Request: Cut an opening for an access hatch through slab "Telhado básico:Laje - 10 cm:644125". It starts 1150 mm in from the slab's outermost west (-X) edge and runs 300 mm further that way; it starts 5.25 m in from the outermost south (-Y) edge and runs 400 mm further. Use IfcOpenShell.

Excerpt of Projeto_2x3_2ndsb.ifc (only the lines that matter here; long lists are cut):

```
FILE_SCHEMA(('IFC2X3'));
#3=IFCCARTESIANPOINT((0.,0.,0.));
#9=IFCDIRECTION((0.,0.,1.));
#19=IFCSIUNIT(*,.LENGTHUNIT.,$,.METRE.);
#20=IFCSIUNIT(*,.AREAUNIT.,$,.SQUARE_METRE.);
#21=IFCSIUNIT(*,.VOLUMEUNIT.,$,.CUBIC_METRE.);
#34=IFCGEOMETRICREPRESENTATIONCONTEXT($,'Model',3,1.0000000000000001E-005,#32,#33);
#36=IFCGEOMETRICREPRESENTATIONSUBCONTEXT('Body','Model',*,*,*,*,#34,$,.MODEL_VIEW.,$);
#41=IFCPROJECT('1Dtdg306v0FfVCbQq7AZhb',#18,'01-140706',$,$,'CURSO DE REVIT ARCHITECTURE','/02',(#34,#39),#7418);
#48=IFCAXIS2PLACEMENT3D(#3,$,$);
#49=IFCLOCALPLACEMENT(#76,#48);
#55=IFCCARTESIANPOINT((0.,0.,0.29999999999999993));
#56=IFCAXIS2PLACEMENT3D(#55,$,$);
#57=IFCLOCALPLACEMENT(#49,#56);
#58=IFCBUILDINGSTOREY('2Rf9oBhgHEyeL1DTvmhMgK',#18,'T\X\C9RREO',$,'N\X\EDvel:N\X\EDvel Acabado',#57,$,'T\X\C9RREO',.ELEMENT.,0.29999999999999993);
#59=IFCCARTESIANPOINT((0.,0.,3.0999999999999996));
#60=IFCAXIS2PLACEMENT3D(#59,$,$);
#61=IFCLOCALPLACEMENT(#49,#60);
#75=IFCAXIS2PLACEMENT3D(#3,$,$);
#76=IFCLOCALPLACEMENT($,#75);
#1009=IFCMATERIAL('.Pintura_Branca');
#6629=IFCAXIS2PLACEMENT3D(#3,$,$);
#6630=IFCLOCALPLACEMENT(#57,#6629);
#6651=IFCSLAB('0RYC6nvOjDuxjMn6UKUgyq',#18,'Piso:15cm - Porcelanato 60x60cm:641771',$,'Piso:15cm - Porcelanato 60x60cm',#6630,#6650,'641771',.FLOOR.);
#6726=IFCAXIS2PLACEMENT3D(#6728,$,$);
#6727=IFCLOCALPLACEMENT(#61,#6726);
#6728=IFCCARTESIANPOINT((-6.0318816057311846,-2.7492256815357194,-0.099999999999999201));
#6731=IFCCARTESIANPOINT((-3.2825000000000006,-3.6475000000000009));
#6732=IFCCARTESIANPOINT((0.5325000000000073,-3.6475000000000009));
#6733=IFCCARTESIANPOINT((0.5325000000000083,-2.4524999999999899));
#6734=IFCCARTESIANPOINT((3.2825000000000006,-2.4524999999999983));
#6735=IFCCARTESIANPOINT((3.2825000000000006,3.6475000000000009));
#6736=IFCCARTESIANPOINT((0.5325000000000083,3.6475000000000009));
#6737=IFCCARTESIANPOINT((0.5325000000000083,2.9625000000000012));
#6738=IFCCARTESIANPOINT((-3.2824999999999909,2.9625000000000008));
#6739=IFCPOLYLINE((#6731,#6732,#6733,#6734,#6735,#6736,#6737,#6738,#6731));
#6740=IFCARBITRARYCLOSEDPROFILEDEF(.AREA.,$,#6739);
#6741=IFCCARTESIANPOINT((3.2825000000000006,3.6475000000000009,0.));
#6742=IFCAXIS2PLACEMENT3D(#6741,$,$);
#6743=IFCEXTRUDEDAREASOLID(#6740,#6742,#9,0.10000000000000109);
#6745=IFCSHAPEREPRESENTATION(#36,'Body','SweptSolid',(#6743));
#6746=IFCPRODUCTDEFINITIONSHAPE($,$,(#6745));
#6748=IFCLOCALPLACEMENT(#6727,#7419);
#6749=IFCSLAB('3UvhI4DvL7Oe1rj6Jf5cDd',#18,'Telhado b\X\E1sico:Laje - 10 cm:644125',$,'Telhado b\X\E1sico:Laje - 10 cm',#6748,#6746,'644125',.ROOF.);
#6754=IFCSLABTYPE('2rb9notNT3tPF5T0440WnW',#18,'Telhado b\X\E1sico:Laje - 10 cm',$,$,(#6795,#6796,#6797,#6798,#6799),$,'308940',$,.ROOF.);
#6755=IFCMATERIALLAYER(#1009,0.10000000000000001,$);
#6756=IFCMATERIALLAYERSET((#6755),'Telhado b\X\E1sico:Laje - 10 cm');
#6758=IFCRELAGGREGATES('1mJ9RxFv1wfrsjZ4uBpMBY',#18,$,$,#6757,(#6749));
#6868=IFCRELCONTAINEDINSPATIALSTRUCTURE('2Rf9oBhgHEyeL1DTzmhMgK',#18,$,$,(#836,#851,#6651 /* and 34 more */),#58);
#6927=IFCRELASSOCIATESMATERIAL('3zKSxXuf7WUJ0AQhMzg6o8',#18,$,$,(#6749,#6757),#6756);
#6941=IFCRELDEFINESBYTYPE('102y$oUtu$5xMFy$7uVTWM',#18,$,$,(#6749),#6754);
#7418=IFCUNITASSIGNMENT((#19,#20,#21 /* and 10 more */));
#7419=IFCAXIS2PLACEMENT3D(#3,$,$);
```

```python
import numpy as np
import ifcopenshell
import ifcopenshell.api.feature
import ifcopenshell.api.geometry
import ifcopenshell.api.root
import ifcopenshell.geom
import ifcopenshell.util.placement
import ifcopenshell.util.representation
import ifcopenshell.util.shape
import ifcopenshell.util.unit

model = ifcopenshell.open("Projeto_2x3_2ndsb.ifc")
unit_scale = ifcopenshell.util.unit.calculate_unit_scale(model)
settings = ifcopenshell.geom.settings()


def volume(element):
    """Net volume in cubic metres, openings subtracted."""
    shape = ifcopenshell.geom.create_shape(settings, element)
    return ifcopenshell.util.shape.get_volume(shape.geometry)


slab = model.by_guid("3UvhI4DvL7Oe1rj6Jf5cDd")
before = volume(slab)

# Extent in the slab's own axes, in metres. The edges named are its -X and -Y sides.
slab_shape = ifcopenshell.geom.create_shape(settings, slab)
vertices = ifcopenshell.util.shape.get_vertices(slab_shape.geometry)
x_min, y_min, bottom = vertices.min(axis=0)
top = vertices[:, 2].max()

opening = ifcopenshell.api.root.create_entity(model, ifc_class="IfcOpeningElement", name="Access hatch opening")
context = ifcopenshell.util.representation.get_context(model, "Model", "Body", "MODEL_VIEW")
width, depth = 0.3, 0.4
outline = [(0.0, 0.0), (width, 0.0), (width, depth), (0.0, depth), (0.0, 0.0)]
# Overshoot both faces by 50 mm so the cut is clean.
shape = ifcopenshell.api.geometry.add_slab_representation(
    model, context=context, depth=top - bottom + 0.1, polyline=outline
)
ifcopenshell.api.geometry.assign_representation(model, product=opening, representation=shape)

matrix = ifcopenshell.util.placement.get_local_placement(slab.ObjectPlacement)
matrix[:, 3] = matrix @ np.append(np.array([x_min + 1.15, y_min + 5.25, bottom - 0.05]) / unit_scale, 1.0)
ifcopenshell.api.geometry.edit_object_placement(model, product=opening, matrix=matrix, is_si=False)
ifcopenshell.api.feature.add_feature(model, feature=opening, element=slab)

after = volume(slab)

print(f"slab volume {before:.3f} -> {after:.3f} m3")

model.write("Projeto_2x3_2ndsb_v2.ifc")
```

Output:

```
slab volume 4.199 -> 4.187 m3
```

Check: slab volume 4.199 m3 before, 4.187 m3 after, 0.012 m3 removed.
